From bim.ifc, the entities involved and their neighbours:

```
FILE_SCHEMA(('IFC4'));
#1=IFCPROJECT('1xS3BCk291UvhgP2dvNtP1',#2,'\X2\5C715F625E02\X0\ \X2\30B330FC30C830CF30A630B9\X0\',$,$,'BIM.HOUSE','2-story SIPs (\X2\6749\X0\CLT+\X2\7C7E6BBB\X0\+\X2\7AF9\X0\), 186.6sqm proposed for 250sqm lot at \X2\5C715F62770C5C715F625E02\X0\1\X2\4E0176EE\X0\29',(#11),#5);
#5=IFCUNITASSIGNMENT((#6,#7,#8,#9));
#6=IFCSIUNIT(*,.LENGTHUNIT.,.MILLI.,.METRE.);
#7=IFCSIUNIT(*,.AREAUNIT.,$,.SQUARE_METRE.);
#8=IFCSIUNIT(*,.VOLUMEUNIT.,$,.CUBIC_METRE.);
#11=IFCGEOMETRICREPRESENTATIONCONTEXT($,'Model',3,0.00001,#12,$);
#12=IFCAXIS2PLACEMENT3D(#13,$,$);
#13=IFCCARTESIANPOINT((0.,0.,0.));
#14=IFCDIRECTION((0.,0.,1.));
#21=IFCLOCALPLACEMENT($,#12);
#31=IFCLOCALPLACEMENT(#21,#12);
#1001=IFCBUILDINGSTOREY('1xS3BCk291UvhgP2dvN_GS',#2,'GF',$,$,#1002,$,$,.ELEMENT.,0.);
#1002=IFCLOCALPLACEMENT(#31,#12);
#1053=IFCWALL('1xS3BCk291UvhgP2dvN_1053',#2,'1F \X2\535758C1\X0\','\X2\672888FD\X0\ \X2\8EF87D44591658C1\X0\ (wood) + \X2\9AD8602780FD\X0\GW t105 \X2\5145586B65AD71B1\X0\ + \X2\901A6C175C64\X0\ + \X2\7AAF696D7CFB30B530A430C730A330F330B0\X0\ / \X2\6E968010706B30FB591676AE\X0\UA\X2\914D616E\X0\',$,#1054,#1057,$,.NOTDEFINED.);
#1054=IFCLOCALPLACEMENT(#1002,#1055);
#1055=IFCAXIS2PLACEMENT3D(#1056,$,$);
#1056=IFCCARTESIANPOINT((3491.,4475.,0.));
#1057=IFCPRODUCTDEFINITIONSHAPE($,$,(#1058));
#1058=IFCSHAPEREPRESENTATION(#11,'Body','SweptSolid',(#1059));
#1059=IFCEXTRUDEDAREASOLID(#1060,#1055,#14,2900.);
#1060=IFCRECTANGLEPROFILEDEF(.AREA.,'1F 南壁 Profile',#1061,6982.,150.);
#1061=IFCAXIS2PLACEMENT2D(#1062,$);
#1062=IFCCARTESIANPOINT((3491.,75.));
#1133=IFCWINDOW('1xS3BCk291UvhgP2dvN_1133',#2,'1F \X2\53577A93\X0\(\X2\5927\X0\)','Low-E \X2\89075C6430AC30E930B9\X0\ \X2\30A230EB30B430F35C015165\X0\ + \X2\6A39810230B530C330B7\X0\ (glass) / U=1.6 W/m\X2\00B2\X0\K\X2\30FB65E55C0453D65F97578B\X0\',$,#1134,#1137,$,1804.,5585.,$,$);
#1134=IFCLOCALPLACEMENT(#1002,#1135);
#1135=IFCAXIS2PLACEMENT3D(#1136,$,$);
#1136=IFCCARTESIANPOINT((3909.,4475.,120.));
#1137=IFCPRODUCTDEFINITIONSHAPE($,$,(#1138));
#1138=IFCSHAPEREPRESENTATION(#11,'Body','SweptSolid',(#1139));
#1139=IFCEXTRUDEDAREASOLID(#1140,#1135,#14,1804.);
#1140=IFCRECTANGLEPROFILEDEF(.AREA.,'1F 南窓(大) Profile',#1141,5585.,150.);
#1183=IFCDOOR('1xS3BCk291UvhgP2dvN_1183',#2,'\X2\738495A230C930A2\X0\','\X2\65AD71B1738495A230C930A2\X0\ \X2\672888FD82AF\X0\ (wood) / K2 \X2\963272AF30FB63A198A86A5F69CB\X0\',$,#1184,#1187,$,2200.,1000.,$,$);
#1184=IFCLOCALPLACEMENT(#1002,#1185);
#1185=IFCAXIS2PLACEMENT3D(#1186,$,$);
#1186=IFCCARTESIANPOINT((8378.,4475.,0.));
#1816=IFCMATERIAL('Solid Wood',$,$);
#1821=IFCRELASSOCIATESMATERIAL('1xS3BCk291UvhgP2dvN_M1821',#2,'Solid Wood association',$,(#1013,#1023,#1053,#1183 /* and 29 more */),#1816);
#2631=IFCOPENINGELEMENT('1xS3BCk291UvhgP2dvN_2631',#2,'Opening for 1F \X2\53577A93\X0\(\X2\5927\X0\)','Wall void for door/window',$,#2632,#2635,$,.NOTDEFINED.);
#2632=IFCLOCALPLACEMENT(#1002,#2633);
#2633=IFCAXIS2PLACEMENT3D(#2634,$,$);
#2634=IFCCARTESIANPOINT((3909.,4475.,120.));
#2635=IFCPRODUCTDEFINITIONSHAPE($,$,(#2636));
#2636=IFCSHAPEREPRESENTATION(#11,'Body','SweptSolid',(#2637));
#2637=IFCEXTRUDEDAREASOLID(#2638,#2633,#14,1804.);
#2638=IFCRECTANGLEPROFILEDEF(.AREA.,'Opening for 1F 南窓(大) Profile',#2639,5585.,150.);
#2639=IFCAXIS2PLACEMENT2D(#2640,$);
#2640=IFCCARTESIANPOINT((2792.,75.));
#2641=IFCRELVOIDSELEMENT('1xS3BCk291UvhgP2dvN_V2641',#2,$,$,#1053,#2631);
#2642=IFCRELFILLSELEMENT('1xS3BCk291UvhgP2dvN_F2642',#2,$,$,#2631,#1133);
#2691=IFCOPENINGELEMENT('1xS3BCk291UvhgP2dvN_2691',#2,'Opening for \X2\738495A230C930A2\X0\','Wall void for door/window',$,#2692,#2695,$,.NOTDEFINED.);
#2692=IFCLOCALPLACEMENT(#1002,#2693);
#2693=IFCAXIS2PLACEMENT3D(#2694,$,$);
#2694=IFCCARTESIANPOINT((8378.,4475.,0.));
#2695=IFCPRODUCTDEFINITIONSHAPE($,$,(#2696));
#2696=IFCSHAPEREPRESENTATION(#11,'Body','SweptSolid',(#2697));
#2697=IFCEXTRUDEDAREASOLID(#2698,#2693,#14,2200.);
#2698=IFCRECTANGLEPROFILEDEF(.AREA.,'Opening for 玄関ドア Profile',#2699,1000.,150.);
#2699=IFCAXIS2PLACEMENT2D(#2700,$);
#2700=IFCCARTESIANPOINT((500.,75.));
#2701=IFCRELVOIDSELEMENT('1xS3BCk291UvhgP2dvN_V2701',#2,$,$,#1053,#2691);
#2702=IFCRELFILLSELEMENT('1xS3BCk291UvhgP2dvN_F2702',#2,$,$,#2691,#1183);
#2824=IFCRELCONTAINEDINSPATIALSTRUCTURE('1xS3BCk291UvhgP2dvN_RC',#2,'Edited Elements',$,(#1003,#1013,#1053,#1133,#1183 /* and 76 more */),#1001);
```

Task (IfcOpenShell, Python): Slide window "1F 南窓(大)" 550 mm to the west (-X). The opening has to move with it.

```python
import ifcopenshell
import ifcopenshell.api.geometry
import ifcopenshell.util.placement
import ifcopenshell.util.unit

model = ifcopenshell.open("bim.ifc")
unit_scale = ifcopenshell.util.unit.calculate_unit_scale(model)

window = model.by_guid("1xS3BCk291UvhgP2dvN_1133")
opening = window.FillsVoids[0].RelatingOpeningElement
wall = opening.VoidsElements[0].RelatingBuildingElement

wall_matrix = ifcopenshell.util.placement.get_local_placement(wall.ObjectPlacement)
shift = wall_matrix[:3, 0] * -0.55 / unit_scale
before = ifcopenshell.util.placement.get_local_placement(window.ObjectPlacement)[:3, 3].copy()

# The window is not placed relative to its opening, so move both.
for product in (opening, window):
    matrix = ifcopenshell.util.placement.get_local_placement(product.ObjectPlacement)
    matrix[:3, 3] += shift
    ifcopenshell.api.geometry.edit_object_placement(model, product=product, matrix=matrix, is_si=False)

after = ifcopenshell.util.placement.get_local_placement(window.ObjectPlacement)[:3, 3]
print("window moved by", (after - before).round(3) + 0.0)

model.write("bim_edited.ifc")
```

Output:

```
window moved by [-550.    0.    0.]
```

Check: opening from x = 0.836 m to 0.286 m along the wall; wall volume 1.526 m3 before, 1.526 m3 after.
